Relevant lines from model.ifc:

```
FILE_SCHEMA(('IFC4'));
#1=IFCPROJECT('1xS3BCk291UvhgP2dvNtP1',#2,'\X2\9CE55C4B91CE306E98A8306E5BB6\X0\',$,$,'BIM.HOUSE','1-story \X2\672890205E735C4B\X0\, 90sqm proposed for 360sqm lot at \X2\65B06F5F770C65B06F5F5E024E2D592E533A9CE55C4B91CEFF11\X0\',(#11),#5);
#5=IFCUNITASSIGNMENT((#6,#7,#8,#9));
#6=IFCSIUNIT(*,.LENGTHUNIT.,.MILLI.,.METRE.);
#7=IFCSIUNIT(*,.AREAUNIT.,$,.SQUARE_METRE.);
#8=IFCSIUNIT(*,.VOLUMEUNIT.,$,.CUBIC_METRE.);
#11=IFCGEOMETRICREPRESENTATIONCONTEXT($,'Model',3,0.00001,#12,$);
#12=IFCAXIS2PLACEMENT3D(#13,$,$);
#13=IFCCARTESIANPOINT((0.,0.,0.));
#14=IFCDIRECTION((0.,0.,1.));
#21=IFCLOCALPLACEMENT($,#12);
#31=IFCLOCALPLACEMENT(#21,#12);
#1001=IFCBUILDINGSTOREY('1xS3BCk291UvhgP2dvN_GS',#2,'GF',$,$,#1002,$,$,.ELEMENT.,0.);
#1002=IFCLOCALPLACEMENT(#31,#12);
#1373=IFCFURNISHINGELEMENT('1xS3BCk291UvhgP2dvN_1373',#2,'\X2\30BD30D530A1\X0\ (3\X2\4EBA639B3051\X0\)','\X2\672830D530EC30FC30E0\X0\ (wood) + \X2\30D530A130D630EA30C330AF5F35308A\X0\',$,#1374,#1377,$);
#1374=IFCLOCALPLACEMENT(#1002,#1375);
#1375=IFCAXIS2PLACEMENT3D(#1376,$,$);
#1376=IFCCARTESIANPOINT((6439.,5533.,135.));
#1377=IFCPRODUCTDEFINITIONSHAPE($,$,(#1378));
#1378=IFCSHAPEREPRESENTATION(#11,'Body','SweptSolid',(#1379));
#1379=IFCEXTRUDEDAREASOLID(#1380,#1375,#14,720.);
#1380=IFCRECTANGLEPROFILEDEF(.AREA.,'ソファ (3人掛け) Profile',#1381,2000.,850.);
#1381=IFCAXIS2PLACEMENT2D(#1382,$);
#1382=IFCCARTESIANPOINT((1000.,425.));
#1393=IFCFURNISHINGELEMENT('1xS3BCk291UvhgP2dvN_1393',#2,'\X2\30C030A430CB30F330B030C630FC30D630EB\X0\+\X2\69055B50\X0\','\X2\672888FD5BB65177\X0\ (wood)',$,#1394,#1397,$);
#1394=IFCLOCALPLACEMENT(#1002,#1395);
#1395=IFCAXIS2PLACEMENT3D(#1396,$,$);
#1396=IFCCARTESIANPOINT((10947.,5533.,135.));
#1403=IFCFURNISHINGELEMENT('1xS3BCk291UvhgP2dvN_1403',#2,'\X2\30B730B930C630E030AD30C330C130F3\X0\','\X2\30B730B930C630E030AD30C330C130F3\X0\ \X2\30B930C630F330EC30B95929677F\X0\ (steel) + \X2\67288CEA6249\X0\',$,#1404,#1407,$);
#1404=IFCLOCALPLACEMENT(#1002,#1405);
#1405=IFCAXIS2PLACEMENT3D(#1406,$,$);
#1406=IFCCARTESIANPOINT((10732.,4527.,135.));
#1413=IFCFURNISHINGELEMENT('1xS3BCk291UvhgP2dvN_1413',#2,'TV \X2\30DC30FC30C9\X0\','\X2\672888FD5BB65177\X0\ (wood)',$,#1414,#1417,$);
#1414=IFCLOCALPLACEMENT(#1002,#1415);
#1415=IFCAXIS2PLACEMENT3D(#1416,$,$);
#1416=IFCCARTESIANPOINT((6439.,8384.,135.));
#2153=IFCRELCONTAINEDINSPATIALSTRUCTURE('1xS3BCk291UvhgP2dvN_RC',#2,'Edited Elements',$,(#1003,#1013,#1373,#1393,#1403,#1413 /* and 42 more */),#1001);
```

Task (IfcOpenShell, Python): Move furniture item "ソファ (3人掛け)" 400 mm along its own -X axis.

```python
import ifcopenshell
import ifcopenshell.api.geometry
import ifcopenshell.util.placement

model = ifcopenshell.open("model.ifc")

item = model.by_guid("1xS3BCk291UvhgP2dvN_1373")
matrix = ifcopenshell.util.placement.get_local_placement(item.ObjectPlacement)
matrix[:3, 3] -= matrix[:3, 0] * 400.0
ifcopenshell.api.geometry.edit_object_placement(model, product=item, matrix=matrix, is_si=False)

print(ifcopenshell.util.placement.get_local_placement(item.ObjectPlacement).round(3) + 0.0)

model.write("model_v2.ifc")
```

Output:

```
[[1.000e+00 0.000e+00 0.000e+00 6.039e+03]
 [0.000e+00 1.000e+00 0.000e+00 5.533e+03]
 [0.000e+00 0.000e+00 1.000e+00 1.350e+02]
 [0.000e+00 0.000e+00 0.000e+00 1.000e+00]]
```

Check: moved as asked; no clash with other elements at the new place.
